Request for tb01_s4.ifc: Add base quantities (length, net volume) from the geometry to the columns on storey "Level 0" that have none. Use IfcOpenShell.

First a look at what the model holds.

```python
import ifcopenshell
import ifcopenshell.util.element
import ifcopenshell.util.unit

model = ifcopenshell.open("tb01_s4.ifc")
print(model.schema)
for unit_type in ("LENGTHUNIT", "AREAUNIT", "VOLUMEUNIT"):
    print(unit_type, ifcopenshell.util.unit.calculate_unit_scale(model, unit_type))
storey = next(s for s in model.by_type("IfcBuildingStorey") if s.Name == "Level 0")
columns = [e for e in ifcopenshell.util.element.get_decomposition(storey) if e.is_a("IfcColumn")]
for e in sorted(columns, key=lambda e: e.id()):
    print(e.id(), e.is_a(), e.Name, list(ifcopenshell.util.element.get_psets(e, qtos_only=True)), sep=" | ")
```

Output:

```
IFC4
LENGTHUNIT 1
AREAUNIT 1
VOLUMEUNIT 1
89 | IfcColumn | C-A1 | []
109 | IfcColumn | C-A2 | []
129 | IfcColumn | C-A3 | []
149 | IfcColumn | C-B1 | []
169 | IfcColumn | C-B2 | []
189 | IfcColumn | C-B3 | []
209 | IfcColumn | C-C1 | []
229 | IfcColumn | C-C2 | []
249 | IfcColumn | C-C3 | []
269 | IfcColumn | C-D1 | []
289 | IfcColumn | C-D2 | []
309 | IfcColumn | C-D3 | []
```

```python
import ifcopenshell
import ifcopenshell.api.pset
import ifcopenshell.geom
import ifcopenshell.util.element
import ifcopenshell.util.shape
import ifcopenshell.util.unit

model = ifcopenshell.open("tb01_s4.ifc")
unit_scale = ifcopenshell.util.unit.calculate_unit_scale(model)
volume_scale = ifcopenshell.util.unit.calculate_unit_scale(model, "VOLUMEUNIT")
settings = ifcopenshell.geom.settings()

storey = next(s for s in model.by_type("IfcBuildingStorey") if s.Name == "Level 0")
columns = [e for e in ifcopenshell.util.element.get_decomposition(storey) if e.is_a("IfcColumn")]

for e in sorted(columns, key=lambda e: e.id()):
    if ifcopenshell.util.element.get_psets(e, qtos_only=True, should_inherit=False):
        continue
    # Geometry comes back in metres, in the element's own axes.
    shape = ifcopenshell.geom.create_shape(settings, e)
    values = {
        "Length": ifcopenshell.util.shape.get_z(shape.geometry) / unit_scale,
        "NetVolume": ifcopenshell.util.shape.get_volume(shape.geometry) / volume_scale,
    }
    qto = ifcopenshell.api.pset.add_qto(model, product=e, name="Qto_ColumnBaseQuantities")
    ifcopenshell.api.pset.edit_qto(model, qto=qto, properties=values)
    print(e.id(), {k: round(v, 3) for k, v in values.items()})

model.write("tb01_s4_updated.ifc")
```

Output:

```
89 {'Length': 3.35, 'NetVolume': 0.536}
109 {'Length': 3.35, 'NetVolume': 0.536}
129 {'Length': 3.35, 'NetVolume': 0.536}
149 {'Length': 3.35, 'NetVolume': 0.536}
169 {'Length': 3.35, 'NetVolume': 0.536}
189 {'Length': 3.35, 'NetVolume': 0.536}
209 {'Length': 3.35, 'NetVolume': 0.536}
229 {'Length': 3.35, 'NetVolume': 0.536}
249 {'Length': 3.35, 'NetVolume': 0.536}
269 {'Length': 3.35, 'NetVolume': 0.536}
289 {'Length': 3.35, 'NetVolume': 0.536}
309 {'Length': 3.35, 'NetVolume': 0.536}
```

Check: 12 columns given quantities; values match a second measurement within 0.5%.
